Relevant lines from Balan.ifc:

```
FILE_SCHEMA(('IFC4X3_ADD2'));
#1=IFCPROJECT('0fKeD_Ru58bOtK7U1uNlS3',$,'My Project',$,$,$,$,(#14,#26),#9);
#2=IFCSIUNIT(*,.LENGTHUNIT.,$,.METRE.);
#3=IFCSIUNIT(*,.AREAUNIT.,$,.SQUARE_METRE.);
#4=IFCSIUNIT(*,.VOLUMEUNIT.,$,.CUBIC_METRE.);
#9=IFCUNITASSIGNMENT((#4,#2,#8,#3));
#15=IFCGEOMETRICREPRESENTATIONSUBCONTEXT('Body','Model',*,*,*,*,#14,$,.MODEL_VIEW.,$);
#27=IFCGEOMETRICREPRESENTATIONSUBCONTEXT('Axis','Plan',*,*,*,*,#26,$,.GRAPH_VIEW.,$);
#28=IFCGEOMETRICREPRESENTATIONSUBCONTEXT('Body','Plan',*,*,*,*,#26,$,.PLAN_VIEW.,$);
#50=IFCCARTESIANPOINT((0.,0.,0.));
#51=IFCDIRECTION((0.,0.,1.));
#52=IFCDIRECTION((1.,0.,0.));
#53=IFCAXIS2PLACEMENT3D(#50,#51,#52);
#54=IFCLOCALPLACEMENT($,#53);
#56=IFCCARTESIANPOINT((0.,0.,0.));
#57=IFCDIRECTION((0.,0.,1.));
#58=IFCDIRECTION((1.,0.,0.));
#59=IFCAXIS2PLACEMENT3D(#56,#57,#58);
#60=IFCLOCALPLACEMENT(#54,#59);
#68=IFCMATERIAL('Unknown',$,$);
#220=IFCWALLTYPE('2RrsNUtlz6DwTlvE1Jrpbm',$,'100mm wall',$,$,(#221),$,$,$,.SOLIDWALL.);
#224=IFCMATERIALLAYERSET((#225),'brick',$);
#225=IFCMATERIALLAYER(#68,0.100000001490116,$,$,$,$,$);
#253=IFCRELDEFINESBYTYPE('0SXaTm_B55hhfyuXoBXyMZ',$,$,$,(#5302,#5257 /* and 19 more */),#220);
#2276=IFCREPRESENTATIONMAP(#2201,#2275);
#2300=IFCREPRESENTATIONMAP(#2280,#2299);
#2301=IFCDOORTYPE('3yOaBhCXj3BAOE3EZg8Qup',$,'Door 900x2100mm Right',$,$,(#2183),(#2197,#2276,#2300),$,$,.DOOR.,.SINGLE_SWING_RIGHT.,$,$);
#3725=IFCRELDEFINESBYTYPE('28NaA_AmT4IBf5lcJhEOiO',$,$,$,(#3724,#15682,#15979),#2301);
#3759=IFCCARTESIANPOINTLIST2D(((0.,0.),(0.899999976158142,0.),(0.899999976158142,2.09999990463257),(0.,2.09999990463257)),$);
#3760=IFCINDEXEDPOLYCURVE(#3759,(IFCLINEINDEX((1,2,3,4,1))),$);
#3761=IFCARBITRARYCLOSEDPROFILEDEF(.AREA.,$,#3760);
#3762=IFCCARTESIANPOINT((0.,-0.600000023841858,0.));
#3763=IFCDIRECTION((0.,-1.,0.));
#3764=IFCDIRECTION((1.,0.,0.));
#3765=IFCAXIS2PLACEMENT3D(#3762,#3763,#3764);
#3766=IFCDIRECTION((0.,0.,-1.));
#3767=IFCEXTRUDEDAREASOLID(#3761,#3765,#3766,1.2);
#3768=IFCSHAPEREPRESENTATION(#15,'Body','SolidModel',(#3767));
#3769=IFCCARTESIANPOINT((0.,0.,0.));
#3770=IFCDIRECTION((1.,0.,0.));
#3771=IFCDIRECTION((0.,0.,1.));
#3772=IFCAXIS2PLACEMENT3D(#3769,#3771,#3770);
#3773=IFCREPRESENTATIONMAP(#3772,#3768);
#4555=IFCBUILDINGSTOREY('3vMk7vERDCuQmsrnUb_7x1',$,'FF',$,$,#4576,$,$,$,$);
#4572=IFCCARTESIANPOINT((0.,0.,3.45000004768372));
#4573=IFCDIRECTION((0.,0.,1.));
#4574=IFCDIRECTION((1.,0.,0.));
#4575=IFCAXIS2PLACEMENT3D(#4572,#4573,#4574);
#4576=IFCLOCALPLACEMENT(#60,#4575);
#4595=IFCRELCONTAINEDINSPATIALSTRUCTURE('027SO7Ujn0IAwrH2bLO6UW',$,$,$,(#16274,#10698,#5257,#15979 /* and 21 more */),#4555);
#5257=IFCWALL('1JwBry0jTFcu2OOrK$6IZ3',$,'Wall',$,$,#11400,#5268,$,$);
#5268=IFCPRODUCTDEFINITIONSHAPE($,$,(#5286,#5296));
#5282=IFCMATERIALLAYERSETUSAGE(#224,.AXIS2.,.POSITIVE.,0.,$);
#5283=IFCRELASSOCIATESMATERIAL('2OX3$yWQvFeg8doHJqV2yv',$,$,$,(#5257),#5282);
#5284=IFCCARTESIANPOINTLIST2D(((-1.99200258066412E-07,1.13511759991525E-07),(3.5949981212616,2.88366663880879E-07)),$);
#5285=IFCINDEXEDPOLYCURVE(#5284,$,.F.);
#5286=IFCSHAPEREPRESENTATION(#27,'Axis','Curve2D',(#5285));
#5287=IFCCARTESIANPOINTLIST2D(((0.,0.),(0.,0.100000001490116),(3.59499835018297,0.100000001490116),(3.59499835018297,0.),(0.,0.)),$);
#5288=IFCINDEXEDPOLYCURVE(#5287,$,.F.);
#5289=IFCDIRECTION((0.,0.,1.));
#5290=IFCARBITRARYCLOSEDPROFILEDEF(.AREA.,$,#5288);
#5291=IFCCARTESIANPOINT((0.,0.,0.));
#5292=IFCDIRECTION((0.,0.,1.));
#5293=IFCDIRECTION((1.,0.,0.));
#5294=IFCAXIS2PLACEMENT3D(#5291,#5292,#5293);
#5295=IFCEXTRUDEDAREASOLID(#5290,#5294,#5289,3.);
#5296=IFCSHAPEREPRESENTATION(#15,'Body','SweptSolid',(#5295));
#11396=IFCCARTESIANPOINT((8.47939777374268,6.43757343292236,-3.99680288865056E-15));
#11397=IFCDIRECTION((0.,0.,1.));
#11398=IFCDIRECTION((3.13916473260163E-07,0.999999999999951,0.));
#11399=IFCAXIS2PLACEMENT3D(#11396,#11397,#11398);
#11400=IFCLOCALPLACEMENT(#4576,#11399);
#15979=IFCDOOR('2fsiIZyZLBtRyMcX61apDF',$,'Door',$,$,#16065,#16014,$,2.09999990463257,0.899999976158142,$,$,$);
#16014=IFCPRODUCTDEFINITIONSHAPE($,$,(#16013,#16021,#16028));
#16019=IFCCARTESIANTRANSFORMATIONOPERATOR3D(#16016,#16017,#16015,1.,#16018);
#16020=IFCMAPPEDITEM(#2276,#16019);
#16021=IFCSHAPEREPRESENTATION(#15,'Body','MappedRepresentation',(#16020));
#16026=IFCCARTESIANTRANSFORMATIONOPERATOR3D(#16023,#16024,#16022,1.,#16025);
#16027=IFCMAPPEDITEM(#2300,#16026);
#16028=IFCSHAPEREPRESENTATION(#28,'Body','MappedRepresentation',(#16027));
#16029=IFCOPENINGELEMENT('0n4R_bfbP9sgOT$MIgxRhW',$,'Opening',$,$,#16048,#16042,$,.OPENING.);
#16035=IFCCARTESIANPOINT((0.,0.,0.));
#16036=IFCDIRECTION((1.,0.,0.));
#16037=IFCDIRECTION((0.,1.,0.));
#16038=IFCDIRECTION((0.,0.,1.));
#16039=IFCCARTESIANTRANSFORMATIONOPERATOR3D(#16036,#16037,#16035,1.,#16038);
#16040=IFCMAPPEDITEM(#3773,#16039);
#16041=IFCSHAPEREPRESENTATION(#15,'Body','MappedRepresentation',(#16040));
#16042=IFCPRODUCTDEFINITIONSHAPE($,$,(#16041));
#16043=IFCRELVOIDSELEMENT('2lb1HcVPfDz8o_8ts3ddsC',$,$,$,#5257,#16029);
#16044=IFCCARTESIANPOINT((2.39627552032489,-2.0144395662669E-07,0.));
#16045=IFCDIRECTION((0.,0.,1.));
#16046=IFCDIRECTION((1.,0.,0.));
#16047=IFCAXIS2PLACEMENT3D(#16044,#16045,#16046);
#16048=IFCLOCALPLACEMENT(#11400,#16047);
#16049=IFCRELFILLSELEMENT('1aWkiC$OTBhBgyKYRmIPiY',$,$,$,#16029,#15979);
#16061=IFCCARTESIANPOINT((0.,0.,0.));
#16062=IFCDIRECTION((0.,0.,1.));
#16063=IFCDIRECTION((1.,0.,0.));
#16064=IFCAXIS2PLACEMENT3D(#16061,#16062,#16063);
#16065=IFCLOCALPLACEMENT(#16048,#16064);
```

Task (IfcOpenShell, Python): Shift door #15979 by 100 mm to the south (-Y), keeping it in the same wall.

```python
import ifcopenshell
import ifcopenshell.api.geometry
import ifcopenshell.util.placement
import ifcopenshell.util.unit

model = ifcopenshell.open("Balan.ifc")
unit_scale = ifcopenshell.util.unit.calculate_unit_scale(model)

door = model.by_guid("2fsiIZyZLBtRyMcX61apDF")
opening = door.FillsVoids[0].RelatingOpeningElement
wall = opening.VoidsElements[0].RelatingBuildingElement

wall_matrix = ifcopenshell.util.placement.get_local_placement(wall.ObjectPlacement)
shift = wall_matrix[:3, 0] * -0.1 / unit_scale
before = ifcopenshell.util.placement.get_local_placement(door.ObjectPlacement)[:3, 3].copy()

# The door is placed relative to its opening, so it follows when the opening moves.
matrix = ifcopenshell.util.placement.get_local_placement(opening.ObjectPlacement)
matrix[:3, 3] += shift
ifcopenshell.api.geometry.edit_object_placement(
    model, product=opening, matrix=matrix, is_si=False, should_transform_children=True
)

after = ifcopenshell.util.placement.get_local_placement(door.ObjectPlacement)[:3, 3]
print("door moved by", (after - before).round(3) + 0.0)

model.write("Balan-out.ifc")
```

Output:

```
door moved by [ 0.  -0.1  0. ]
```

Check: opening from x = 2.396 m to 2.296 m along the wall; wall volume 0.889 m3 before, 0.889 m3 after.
